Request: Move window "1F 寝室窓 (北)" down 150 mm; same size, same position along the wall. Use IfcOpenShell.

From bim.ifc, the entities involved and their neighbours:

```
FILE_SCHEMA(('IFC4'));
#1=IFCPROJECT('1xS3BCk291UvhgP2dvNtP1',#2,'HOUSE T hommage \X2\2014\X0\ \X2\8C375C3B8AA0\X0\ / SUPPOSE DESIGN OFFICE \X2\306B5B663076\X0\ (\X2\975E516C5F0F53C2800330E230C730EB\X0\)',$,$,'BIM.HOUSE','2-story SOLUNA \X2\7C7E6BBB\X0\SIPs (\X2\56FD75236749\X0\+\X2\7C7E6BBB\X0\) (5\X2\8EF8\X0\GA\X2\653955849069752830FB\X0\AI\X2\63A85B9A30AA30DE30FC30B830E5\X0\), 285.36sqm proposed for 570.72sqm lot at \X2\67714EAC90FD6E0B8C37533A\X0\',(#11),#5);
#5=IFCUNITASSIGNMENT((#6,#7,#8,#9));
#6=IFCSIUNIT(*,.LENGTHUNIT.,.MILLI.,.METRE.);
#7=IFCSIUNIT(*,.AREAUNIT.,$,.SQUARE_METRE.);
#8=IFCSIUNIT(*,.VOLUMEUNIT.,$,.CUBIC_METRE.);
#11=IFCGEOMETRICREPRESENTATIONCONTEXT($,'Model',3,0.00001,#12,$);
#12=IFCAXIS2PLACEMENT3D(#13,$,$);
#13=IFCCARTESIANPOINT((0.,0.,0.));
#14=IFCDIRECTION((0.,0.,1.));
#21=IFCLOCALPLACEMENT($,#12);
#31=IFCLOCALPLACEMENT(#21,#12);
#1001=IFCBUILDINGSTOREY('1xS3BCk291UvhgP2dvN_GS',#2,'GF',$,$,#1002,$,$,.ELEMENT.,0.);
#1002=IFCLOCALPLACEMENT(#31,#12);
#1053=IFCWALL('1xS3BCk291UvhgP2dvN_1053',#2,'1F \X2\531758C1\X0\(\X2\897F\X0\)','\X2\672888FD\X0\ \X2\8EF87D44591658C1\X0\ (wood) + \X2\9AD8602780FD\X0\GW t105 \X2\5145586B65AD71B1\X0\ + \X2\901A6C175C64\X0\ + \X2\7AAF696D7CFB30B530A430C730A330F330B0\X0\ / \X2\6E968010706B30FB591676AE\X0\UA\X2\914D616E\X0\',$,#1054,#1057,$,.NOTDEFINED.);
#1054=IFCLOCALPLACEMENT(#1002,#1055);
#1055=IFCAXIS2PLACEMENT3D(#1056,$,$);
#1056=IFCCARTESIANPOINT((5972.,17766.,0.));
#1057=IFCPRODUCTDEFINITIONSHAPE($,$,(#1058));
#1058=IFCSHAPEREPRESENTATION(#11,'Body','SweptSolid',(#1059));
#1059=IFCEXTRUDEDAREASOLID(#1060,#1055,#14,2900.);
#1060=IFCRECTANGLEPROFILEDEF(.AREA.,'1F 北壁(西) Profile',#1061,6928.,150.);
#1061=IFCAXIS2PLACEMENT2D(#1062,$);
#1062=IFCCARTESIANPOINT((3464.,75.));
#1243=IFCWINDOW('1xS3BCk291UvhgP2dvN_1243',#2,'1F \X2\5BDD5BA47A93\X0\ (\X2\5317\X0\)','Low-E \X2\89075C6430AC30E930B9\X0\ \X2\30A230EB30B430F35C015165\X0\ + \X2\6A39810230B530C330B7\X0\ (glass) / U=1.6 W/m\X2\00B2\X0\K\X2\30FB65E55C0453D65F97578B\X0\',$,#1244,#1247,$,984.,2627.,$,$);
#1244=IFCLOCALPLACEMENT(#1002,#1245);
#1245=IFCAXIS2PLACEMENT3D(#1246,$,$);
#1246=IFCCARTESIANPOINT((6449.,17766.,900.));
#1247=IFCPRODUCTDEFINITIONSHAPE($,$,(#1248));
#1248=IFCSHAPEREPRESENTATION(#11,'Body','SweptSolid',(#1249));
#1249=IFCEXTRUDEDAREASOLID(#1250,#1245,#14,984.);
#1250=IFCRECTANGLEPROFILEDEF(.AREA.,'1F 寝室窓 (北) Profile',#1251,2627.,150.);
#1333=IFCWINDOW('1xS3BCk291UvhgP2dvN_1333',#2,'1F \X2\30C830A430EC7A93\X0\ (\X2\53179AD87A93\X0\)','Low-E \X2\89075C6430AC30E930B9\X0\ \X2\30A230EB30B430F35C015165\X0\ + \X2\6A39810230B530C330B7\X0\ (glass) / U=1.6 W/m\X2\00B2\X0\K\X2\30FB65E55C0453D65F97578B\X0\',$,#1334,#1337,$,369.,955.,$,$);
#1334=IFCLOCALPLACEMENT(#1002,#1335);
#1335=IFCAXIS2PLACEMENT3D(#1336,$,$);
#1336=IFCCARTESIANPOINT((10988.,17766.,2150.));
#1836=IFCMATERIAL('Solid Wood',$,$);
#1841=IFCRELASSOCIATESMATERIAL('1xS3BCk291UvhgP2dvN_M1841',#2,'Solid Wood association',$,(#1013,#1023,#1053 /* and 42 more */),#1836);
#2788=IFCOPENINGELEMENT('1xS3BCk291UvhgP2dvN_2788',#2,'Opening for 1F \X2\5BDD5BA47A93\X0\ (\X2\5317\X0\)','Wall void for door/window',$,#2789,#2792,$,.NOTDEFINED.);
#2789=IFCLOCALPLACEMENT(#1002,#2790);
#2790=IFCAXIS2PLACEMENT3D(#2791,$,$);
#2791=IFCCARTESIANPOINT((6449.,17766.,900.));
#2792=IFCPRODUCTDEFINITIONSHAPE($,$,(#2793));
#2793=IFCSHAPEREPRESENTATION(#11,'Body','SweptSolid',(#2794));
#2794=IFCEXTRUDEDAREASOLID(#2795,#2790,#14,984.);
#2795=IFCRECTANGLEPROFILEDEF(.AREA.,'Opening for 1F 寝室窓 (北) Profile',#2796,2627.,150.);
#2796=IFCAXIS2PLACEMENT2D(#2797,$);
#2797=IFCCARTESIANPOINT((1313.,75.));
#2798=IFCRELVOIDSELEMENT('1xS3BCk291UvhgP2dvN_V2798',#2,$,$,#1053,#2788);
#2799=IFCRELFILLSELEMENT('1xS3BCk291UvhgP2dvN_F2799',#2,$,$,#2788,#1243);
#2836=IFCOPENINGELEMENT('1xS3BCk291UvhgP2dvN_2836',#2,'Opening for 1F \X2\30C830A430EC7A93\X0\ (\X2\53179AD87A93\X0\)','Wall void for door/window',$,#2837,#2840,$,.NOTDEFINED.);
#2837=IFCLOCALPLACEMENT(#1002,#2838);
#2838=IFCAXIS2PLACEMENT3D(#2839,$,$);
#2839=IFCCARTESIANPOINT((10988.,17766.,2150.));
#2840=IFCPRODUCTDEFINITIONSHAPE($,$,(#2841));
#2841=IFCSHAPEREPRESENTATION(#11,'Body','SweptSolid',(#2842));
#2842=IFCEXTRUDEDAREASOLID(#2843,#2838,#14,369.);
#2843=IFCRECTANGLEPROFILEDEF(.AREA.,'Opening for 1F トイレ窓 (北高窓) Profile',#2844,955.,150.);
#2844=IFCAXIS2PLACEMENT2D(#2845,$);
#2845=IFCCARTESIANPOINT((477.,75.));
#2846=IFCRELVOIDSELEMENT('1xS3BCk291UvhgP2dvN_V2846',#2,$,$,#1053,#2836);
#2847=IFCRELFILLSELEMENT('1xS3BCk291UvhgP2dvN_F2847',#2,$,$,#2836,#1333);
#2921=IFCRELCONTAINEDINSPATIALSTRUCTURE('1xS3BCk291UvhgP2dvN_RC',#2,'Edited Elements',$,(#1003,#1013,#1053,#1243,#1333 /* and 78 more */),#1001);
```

```python
import numpy as np
import ifcopenshell
import ifcopenshell.api.geometry
import ifcopenshell.util.placement
import ifcopenshell.util.unit

model = ifcopenshell.open("bim.ifc")
unit_scale = ifcopenshell.util.unit.calculate_unit_scale(model)

window = model.by_guid("1xS3BCk291UvhgP2dvN_1243")
opening = window.FillsVoids[0].RelatingOpeningElement
dz = -150.0

shift = np.array([0.0, 0.0, dz])
# The window is not placed relative to its opening, so move both.
for product in (opening, window):
    matrix = ifcopenshell.util.placement.get_local_placement(product.ObjectPlacement)
    matrix[:3, 3] += shift
    ifcopenshell.api.geometry.edit_object_placement(model, product=product, matrix=matrix, is_si=False)

print(f"moved by {dz * unit_scale:+.3f} m")

model.write("bim_edited.ifc")
```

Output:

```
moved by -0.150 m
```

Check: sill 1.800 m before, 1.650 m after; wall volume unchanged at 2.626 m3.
